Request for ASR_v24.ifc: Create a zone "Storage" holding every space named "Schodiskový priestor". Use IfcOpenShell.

First a look at what the model holds.

```python
import ifcopenshell

model = ifcopenshell.open("ASR_v24.ifc")
print(model.schema)
seen = {}
for space in model.by_type("IfcSpace"):
    seen[space.LongName] = seen.get(space.LongName, 0) + 1
for name, count in sorted(seen.items(), key=str):
    print(count, "x", name)
print("zones:", [z.Name for z in model.by_type("IfcZone")][:20])
```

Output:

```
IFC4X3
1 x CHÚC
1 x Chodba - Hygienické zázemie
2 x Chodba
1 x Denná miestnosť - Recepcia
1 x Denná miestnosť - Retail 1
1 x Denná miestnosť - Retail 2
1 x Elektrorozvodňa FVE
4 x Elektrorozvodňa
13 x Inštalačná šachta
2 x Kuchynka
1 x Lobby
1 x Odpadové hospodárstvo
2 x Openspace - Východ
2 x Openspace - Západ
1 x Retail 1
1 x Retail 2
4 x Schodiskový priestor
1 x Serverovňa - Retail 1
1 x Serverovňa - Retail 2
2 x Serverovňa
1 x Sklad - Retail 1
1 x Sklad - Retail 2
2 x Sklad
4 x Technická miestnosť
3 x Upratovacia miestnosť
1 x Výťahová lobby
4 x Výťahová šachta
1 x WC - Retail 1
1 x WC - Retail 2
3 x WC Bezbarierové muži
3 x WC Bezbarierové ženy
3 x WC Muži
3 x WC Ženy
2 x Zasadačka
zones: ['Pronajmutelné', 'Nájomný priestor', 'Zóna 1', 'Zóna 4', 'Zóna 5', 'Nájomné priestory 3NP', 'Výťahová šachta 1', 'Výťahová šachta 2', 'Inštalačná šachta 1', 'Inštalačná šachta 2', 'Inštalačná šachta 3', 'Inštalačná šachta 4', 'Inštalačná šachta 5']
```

```python
import ifcopenshell
import ifcopenshell.api.group
import ifcopenshell.api.root

model = ifcopenshell.open("ASR_v24.ifc")

names = {"Schodiskový priestor"}
spaces = [s for s in model.by_type("IfcSpace") if s.LongName in names]

zone = ifcopenshell.api.root.create_entity(model, ifc_class="IfcZone", name="Storage")
ifcopenshell.api.group.assign_group(model, products=spaces, group=zone)
print(len(spaces), "spaces in", zone.Name)

model.write("ASR_v24_edited.ifc")
```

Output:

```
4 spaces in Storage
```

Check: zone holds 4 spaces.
